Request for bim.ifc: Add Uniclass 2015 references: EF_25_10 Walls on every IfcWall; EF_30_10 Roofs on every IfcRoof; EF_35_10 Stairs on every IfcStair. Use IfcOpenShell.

First a look at what the model holds.

```python
import ifcopenshell

model = ifcopenshell.open("bim.ifc")
print(model.schema)
print("classifications:", [c.Name for c in model.by_type("IfcClassification")])
for ifc_class in ("IfcDoor", "IfcRoof", "IfcStair", "IfcWall", "IfcWindow"):
    print(ifc_class, len(model.by_type(ifc_class)))
```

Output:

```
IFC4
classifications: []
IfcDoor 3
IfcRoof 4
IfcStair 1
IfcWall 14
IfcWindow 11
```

```python
import ifcopenshell
import ifcopenshell.api.classification

model = ifcopenshell.open("bim.ifc")

system = ifcopenshell.api.classification.add_classification(model, classification="Uniclass 2015")

codes = {
    "IfcWall": ("EF_25_10", "Walls"),
    "IfcRoof": ("EF_30_10", "Roofs"),
    "IfcStair": ("EF_35_10", "Stairs"),
}
for ifc_class, (code, name) in codes.items():
    products = model.by_type(ifc_class)
    ifcopenshell.api.classification.add_reference(
        model, products=products, classification=system, identification=code, name=name
    )
    print(code, len(products))

model.write("bim_v2.ifc")
```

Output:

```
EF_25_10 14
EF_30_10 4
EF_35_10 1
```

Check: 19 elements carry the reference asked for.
